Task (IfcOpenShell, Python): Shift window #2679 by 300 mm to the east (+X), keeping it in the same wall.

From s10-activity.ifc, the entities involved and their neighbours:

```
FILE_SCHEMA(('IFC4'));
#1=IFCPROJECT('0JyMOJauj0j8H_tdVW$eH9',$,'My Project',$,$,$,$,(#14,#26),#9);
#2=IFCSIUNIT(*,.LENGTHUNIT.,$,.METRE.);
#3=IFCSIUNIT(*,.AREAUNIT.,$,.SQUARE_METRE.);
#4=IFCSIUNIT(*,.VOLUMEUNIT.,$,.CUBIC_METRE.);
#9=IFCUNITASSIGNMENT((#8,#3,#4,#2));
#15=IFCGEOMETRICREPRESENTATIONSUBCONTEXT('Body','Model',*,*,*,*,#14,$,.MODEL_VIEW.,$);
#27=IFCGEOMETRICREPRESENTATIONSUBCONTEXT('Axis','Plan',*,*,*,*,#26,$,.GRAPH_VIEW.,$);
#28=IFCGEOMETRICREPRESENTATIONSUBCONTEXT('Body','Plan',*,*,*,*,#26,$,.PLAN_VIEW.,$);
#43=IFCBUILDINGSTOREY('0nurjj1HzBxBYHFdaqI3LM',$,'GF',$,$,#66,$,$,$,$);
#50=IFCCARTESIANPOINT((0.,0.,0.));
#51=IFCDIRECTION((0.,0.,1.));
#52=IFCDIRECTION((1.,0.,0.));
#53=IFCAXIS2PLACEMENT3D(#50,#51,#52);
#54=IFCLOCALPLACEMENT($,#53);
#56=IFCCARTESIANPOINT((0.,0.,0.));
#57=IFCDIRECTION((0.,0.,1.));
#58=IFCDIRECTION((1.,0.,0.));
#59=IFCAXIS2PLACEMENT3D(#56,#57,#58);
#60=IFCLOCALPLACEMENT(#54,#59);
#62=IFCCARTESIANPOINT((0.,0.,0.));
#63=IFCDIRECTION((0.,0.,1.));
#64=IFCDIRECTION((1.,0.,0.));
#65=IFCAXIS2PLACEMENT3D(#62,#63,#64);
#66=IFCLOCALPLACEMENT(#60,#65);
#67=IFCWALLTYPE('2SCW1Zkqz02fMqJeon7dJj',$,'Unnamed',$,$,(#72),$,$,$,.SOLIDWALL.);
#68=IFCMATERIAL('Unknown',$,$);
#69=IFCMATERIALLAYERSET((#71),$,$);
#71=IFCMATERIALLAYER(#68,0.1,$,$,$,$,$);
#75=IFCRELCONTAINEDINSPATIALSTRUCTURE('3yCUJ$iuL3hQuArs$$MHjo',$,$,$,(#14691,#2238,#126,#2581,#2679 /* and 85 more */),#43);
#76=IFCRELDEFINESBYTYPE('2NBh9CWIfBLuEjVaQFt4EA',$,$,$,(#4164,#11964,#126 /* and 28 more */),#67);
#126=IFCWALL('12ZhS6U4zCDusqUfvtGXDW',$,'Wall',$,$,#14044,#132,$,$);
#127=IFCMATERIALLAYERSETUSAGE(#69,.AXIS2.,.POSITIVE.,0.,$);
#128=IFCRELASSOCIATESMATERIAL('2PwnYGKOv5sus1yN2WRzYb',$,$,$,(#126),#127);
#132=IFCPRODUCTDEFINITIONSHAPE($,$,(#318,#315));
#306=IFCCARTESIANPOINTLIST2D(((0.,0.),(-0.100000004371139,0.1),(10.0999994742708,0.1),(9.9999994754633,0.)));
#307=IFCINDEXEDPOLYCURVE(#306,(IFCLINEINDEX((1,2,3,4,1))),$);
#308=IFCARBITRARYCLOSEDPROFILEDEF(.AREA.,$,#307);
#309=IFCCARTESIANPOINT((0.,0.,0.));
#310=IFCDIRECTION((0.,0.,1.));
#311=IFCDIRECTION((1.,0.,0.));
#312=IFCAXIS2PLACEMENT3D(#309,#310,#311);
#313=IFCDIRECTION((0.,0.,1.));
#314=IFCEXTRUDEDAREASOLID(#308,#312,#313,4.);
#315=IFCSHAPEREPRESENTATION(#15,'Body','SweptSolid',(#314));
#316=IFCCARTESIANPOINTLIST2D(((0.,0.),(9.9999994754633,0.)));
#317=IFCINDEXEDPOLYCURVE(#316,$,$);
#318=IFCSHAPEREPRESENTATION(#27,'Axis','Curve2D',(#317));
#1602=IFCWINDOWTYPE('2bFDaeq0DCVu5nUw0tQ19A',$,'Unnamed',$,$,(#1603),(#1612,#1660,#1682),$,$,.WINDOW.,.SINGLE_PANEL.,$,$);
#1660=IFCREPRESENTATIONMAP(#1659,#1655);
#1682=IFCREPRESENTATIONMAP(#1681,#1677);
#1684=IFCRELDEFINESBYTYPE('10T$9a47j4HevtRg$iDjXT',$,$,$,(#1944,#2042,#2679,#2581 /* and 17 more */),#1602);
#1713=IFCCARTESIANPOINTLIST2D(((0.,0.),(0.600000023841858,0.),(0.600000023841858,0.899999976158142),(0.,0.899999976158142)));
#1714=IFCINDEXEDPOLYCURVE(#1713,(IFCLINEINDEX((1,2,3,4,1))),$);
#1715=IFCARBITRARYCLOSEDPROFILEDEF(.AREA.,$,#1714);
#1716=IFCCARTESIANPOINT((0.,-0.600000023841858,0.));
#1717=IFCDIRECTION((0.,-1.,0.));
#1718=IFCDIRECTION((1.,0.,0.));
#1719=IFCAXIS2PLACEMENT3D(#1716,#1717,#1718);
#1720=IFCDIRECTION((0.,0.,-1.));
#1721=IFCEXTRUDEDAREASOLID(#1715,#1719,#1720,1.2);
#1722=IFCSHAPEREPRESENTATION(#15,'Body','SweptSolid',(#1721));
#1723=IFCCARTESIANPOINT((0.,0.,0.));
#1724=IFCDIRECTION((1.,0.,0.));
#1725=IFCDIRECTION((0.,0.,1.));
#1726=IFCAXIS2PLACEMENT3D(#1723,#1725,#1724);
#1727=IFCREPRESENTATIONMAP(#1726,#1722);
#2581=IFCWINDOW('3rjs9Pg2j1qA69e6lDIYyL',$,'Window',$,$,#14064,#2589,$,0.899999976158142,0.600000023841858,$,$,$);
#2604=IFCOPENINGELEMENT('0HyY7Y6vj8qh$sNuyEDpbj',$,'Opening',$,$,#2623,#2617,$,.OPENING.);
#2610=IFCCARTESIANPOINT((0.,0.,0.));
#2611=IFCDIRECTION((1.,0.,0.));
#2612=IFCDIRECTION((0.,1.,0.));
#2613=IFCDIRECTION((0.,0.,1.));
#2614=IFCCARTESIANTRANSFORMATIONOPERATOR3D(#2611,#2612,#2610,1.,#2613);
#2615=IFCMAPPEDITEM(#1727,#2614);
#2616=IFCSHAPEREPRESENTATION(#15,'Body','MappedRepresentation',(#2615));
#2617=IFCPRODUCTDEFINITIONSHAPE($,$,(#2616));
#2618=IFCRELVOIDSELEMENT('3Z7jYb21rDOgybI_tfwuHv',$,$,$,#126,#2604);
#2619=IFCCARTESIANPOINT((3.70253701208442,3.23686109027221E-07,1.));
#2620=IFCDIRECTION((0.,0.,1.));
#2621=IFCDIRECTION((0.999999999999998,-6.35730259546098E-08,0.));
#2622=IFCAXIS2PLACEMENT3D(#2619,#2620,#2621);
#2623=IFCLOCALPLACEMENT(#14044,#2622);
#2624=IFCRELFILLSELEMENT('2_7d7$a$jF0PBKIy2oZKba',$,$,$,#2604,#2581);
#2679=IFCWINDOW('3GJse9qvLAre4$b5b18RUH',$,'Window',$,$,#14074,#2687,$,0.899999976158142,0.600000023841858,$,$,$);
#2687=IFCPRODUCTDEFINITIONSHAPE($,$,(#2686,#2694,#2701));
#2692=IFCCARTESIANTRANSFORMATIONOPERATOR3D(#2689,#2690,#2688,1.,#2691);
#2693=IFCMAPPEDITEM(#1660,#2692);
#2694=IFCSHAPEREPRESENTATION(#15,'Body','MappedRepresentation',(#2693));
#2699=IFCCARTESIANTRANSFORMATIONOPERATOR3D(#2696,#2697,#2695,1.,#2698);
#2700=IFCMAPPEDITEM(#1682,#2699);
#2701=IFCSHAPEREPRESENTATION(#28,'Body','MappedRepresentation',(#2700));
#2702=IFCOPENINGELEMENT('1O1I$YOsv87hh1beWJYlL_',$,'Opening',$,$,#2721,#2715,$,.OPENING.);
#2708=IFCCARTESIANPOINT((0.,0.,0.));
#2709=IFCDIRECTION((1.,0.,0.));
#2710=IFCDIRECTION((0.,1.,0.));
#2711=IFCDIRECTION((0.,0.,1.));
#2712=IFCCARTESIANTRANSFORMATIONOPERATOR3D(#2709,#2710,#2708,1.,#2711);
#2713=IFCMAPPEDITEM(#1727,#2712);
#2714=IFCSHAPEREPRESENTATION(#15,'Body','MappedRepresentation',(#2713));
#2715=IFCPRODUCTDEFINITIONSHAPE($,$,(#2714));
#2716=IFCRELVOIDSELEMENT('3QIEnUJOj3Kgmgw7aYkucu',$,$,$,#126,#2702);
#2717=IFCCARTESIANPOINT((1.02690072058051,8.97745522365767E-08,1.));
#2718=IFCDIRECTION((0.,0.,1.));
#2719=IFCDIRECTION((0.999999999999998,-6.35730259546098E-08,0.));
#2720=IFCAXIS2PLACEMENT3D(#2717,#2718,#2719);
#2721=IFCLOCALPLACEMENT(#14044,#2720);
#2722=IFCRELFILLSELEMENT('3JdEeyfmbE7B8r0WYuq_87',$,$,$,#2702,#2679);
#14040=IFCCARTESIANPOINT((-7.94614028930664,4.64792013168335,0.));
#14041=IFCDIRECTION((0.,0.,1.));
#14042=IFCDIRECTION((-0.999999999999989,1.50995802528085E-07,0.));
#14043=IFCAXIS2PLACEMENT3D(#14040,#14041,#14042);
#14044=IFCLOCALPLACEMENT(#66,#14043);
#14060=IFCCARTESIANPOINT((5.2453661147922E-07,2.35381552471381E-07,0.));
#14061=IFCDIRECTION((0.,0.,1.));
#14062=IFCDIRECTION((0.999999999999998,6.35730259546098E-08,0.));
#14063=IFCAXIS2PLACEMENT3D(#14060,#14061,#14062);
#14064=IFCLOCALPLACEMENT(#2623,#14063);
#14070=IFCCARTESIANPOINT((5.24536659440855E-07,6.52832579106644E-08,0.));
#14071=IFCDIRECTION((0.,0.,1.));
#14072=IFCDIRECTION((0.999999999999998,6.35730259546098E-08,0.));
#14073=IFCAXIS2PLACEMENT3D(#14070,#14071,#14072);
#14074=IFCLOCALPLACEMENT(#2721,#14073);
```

```python
import ifcopenshell
import ifcopenshell.api.geometry
import ifcopenshell.util.placement
import ifcopenshell.util.unit

model = ifcopenshell.open("s10-activity.ifc")
unit_scale = ifcopenshell.util.unit.calculate_unit_scale(model)

window = model.by_id(2679)
opening = window.FillsVoids[0].RelatingOpeningElement
wall = opening.VoidsElements[0].RelatingBuildingElement

wall_matrix = ifcopenshell.util.placement.get_local_placement(wall.ObjectPlacement)
shift = wall_matrix[:3, 0] * -0.3 / unit_scale
before = ifcopenshell.util.placement.get_local_placement(window.ObjectPlacement)[:3, 3].copy()

# The window is placed relative to its opening, so it follows when the opening moves.
matrix = ifcopenshell.util.placement.get_local_placement(opening.ObjectPlacement)
matrix[:3, 3] += shift
ifcopenshell.api.geometry.edit_object_placement(
    model, product=opening, matrix=matrix, is_si=False, should_transform_children=True
)

after = ifcopenshell.util.placement.get_local_placement(window.ObjectPlacement)[:3, 3]
print("window moved by", (after - before).round(3) + 0.0)

model.write("s10-activity_edited.ifc")
```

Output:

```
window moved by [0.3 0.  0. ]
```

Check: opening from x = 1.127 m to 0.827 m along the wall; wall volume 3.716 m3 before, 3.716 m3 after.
